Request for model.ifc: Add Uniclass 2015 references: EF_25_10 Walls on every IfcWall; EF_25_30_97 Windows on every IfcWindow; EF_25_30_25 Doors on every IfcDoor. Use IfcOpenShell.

First a look at what the model holds.

```python
import ifcopenshell

model = ifcopenshell.open("model.ifc")
print(model.schema)
print("classifications:", [c.Name for c in model.by_type("IfcClassification")])
for ifc_class in ("IfcDoor", "IfcRoof", "IfcStair", "IfcWall", "IfcWindow"):
    print(ifc_class, len(model.by_type(ifc_class)))
```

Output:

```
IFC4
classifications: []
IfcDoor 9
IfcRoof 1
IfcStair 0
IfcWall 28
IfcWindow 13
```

```python
import ifcopenshell
import ifcopenshell.api.classification

model = ifcopenshell.open("model.ifc")

system = ifcopenshell.api.classification.add_classification(model, classification="Uniclass 2015")

codes = {
    "IfcWall": ("EF_25_10", "Walls"),
    "IfcWindow": ("EF_25_30_97", "Windows"),
    "IfcDoor": ("EF_25_30_25", "Doors"),
}
for ifc_class, (code, name) in codes.items():
    products = model.by_type(ifc_class)
    ifcopenshell.api.classification.add_reference(
        model, products=products, classification=system, identification=code, name=name
    )
    print(code, len(products))

model.write("model_rev.ifc")
```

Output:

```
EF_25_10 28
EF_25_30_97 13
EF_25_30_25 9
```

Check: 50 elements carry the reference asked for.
